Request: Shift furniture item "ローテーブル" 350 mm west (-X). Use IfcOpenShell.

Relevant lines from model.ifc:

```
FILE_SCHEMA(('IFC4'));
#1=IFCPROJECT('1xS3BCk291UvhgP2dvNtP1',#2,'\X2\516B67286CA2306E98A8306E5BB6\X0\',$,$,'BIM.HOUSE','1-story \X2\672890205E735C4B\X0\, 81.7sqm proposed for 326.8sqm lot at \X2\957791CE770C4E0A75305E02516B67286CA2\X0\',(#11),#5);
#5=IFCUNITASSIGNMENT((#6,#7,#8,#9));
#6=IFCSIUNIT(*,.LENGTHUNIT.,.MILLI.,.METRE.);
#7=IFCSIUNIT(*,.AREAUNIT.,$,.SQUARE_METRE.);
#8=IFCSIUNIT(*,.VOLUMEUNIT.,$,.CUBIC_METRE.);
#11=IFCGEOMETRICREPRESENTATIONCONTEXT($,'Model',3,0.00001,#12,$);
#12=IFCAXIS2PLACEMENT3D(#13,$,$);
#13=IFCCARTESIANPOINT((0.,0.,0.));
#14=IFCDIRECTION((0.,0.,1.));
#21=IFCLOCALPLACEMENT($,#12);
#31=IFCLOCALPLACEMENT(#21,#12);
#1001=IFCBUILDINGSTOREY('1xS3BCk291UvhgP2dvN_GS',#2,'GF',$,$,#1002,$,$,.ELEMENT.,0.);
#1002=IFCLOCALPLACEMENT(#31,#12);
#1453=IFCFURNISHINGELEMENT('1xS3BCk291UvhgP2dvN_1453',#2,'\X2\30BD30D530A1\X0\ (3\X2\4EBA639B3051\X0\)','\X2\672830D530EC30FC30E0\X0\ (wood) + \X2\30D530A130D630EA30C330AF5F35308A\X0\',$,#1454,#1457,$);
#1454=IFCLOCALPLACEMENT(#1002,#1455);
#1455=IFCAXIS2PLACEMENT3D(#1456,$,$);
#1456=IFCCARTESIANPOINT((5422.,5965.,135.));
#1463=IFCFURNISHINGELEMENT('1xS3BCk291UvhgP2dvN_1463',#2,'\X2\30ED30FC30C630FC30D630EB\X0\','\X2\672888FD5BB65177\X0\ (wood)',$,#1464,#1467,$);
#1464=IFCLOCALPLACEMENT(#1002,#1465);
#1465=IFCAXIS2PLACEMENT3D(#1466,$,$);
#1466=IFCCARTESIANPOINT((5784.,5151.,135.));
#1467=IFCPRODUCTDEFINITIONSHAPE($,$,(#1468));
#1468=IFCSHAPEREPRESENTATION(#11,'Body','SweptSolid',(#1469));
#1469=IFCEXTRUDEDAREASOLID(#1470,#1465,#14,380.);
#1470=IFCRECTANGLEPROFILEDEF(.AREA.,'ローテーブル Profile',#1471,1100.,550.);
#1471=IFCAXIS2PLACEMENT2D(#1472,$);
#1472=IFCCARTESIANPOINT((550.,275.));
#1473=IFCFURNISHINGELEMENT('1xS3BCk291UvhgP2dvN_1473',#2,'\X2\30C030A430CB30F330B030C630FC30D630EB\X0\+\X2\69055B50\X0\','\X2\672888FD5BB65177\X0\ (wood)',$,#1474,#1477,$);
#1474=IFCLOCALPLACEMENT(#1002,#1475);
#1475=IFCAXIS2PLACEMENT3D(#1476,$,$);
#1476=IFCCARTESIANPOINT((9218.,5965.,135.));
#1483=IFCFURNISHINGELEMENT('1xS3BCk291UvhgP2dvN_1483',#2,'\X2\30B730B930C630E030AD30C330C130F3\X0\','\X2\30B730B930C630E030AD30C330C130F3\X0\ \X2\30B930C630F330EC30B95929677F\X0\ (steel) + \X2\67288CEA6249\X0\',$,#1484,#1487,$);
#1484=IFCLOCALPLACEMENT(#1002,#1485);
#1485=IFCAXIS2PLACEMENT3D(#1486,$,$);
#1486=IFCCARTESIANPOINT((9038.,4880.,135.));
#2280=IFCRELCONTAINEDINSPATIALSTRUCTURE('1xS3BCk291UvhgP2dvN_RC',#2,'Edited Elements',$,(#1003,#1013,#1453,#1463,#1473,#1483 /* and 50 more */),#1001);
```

```python
import ifcopenshell
import ifcopenshell.api.geometry
import ifcopenshell.util.placement

model = ifcopenshell.open("model.ifc")

item = model.by_guid("1xS3BCk291UvhgP2dvN_1463")
matrix = ifcopenshell.util.placement.get_local_placement(item.ObjectPlacement)
matrix[0, 3] -= 350.0
ifcopenshell.api.geometry.edit_object_placement(model, product=item, matrix=matrix, is_si=False)

print(ifcopenshell.util.placement.get_local_placement(item.ObjectPlacement).round(3) + 0.0)

model.write("model_updated.ifc")
```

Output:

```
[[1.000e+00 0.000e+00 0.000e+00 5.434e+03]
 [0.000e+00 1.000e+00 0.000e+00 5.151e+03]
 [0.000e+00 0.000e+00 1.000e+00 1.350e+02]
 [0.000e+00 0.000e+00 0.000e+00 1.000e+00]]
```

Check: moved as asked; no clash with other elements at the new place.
